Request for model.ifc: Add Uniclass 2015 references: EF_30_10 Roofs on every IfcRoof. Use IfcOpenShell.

First a look at what the model holds.

```python
import ifcopenshell

model = ifcopenshell.open("model.ifc")
print(model.schema)
print("classifications:", [c.Name for c in model.by_type("IfcClassification")])
for ifc_class in ("IfcDoor", "IfcRoof", "IfcStair", "IfcWall", "IfcWindow"):
    print(ifc_class, len(model.by_type(ifc_class)))
```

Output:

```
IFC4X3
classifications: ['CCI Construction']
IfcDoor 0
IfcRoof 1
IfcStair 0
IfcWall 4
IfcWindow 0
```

```python
import ifcopenshell
import ifcopenshell.api.classification

model = ifcopenshell.open("model.ifc")

system = ifcopenshell.api.classification.add_classification(model, classification="Uniclass 2015")

codes = {
    "IfcRoof": ("EF_30_10", "Roofs"),
}
for ifc_class, (code, name) in codes.items():
    products = model.by_type(ifc_class)
    ifcopenshell.api.classification.add_reference(
        model, products=products, classification=system, identification=code, name=name
    )
    print(code, len(products))

model.write("model-out.ifc")
```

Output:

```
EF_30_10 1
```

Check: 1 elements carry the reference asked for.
